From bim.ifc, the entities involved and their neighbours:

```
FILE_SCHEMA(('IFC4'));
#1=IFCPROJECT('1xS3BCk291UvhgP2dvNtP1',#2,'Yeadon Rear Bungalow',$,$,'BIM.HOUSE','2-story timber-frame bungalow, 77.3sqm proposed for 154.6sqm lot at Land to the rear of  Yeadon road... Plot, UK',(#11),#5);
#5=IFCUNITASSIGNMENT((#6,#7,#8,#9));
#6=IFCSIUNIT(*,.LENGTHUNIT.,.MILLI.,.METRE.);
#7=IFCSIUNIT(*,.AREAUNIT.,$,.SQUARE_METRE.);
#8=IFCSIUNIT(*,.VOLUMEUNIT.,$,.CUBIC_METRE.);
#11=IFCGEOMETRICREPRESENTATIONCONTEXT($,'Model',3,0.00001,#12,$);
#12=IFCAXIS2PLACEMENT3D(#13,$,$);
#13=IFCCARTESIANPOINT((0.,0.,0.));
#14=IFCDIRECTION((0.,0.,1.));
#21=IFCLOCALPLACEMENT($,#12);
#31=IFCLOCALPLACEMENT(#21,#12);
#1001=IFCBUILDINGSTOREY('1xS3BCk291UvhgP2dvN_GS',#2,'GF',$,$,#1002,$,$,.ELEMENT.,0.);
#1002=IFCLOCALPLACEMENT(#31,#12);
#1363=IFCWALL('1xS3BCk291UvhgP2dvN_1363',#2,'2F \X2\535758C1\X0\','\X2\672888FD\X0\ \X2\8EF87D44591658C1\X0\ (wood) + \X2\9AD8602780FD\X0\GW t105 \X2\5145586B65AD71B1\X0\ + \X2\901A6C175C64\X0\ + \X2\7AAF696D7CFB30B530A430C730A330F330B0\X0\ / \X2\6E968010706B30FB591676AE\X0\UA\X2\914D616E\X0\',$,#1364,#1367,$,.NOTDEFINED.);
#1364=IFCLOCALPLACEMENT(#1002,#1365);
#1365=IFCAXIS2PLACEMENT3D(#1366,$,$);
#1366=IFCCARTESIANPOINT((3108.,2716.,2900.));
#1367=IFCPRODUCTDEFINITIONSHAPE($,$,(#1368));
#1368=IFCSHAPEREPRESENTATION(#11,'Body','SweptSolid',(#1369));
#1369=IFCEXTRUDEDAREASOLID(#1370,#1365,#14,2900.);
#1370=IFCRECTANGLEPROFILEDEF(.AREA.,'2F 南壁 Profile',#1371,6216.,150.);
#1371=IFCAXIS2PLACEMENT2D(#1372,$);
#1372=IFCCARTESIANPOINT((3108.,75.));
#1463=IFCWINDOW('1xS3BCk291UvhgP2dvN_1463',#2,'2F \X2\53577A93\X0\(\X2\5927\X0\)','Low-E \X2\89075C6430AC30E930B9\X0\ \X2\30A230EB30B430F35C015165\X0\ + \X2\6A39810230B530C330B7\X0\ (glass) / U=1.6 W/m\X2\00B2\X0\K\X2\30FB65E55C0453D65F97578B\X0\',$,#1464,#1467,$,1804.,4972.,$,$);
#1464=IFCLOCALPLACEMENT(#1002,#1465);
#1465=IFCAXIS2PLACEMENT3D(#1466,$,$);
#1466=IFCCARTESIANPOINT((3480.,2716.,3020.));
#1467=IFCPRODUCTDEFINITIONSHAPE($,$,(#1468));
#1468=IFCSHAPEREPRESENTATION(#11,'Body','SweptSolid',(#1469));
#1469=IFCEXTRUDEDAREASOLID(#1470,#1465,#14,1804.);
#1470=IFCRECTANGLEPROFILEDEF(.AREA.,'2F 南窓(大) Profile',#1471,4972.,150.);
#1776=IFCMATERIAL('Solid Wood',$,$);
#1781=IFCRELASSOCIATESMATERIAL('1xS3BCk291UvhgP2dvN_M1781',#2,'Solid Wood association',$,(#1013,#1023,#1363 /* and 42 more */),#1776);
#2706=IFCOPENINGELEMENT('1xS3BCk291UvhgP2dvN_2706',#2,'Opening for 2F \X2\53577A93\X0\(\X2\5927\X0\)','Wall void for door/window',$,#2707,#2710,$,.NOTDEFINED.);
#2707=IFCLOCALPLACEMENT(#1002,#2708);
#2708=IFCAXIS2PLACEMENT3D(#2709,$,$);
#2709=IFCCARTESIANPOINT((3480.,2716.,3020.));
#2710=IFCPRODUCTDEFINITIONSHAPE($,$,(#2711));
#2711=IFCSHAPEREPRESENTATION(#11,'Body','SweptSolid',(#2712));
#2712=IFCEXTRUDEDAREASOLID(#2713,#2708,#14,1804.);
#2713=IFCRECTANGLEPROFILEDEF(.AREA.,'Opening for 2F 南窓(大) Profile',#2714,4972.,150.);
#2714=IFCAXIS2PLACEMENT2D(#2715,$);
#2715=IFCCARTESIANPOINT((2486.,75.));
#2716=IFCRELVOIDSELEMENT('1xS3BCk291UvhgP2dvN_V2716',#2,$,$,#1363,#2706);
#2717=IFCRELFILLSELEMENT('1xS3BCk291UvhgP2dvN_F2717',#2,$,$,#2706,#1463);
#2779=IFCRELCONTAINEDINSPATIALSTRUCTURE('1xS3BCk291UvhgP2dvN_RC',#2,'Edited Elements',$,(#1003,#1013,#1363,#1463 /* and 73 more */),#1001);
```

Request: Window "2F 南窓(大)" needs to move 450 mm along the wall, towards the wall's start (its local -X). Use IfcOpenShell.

```python
import ifcopenshell
import ifcopenshell.api.geometry
import ifcopenshell.util.placement
import ifcopenshell.util.unit

model = ifcopenshell.open("bim.ifc")
unit_scale = ifcopenshell.util.unit.calculate_unit_scale(model)

window = model.by_id(1463)
opening = window.FillsVoids[0].RelatingOpeningElement
wall = opening.VoidsElements[0].RelatingBuildingElement

wall_matrix = ifcopenshell.util.placement.get_local_placement(wall.ObjectPlacement)
shift = wall_matrix[:3, 0] * -0.45 / unit_scale
before = ifcopenshell.util.placement.get_local_placement(window.ObjectPlacement)[:3, 3].copy()

# The window is not placed relative to its opening, so move both.
for product in (opening, window):
    matrix = ifcopenshell.util.placement.get_local_placement(product.ObjectPlacement)
    matrix[:3, 3] += shift
    ifcopenshell.api.geometry.edit_object_placement(model, product=product, matrix=matrix, is_si=False)

after = ifcopenshell.util.placement.get_local_placement(window.ObjectPlacement)[:3, 3]
print("window moved by", (after - before).round(3) + 0.0)

model.write("bim-out.ifc")
```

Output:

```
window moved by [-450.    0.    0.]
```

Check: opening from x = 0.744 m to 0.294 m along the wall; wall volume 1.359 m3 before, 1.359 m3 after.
